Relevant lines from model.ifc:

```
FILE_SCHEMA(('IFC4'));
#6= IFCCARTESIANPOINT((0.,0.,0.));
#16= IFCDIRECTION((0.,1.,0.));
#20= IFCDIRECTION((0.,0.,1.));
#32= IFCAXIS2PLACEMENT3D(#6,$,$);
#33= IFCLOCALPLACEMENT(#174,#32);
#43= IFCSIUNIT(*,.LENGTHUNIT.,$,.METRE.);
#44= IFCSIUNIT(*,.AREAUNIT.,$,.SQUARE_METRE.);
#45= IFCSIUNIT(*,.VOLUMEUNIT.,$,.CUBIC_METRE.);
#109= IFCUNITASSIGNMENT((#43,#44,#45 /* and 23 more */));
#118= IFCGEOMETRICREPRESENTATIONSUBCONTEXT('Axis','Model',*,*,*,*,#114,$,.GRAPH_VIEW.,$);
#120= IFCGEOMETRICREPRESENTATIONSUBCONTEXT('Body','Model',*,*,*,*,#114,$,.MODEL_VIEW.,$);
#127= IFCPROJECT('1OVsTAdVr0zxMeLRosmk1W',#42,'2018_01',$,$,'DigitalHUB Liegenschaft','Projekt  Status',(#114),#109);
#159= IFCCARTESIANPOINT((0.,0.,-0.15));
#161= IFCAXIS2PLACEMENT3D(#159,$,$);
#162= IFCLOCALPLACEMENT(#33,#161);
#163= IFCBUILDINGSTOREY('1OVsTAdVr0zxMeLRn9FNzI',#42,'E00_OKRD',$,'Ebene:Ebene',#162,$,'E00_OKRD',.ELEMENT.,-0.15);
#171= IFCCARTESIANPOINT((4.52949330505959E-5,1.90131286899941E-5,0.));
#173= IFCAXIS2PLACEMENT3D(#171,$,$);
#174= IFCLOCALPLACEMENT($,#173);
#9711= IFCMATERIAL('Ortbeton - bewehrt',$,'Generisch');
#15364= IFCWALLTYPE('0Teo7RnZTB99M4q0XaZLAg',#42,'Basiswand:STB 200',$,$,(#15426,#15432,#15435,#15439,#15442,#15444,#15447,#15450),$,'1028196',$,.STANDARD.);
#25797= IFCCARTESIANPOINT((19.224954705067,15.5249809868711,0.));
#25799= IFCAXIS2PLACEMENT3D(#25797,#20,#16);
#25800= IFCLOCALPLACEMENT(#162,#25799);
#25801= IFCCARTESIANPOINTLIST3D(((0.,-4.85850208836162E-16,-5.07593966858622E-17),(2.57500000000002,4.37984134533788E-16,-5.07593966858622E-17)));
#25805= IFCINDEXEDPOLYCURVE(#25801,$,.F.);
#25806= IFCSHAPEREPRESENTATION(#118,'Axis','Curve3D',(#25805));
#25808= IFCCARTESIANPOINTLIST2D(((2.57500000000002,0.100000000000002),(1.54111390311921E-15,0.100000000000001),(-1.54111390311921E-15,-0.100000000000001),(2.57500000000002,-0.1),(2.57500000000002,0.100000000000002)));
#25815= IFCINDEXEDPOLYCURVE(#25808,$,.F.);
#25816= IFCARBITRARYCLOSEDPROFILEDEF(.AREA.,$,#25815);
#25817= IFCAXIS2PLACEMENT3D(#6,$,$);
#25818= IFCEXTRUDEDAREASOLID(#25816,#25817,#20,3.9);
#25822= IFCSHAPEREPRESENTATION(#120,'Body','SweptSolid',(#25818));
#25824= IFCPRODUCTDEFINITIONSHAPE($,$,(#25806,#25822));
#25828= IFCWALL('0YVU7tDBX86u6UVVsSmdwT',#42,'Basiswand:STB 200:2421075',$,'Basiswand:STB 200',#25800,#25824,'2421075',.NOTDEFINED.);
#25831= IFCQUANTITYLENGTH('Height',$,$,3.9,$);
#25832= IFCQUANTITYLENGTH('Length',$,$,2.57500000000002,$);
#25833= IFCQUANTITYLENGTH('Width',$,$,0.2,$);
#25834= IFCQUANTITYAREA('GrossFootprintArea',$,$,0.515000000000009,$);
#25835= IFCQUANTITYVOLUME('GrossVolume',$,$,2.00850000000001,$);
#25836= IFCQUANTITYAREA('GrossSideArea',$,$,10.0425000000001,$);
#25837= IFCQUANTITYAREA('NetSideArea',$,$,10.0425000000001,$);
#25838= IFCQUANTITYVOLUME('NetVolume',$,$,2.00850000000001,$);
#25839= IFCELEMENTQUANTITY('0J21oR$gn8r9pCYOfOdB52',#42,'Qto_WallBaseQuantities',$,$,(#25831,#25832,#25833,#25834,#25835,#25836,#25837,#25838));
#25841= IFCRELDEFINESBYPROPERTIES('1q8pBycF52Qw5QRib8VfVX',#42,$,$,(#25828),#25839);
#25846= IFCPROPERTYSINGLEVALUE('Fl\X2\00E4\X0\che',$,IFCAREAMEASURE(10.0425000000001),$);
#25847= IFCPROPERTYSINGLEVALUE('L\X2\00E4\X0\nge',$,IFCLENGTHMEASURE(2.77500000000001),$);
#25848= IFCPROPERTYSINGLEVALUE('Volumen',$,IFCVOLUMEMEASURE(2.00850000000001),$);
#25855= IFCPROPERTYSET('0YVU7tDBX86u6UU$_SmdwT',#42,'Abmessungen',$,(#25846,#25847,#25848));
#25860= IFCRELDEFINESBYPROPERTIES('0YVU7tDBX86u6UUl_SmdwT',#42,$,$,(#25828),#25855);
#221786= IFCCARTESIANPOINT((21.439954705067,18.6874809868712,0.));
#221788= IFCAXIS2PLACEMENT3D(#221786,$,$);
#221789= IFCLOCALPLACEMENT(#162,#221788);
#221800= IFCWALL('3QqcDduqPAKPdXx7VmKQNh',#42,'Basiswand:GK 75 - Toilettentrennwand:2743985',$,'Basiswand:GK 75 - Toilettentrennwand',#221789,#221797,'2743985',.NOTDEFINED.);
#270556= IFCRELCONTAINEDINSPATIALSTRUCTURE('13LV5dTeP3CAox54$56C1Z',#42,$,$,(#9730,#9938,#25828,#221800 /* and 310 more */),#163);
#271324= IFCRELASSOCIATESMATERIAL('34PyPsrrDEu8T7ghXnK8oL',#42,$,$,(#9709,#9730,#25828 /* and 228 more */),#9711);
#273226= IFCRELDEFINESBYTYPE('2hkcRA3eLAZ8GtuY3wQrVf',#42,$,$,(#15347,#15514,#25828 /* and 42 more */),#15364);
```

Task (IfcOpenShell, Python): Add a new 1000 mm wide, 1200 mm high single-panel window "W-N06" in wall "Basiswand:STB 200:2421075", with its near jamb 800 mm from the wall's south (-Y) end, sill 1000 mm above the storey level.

```python
import numpy as np
import ifcopenshell
import ifcopenshell.api.feature
import ifcopenshell.api.geometry
import ifcopenshell.api.pset
import ifcopenshell.api.root
import ifcopenshell.api.spatial
import ifcopenshell.geom
import ifcopenshell.util.element
import ifcopenshell.util.placement
import ifcopenshell.util.representation
import ifcopenshell.util.shape
import ifcopenshell.util.unit

model = ifcopenshell.open("model.ifc")
unit_scale = ifcopenshell.util.unit.calculate_unit_scale(model)
area_scale = ifcopenshell.util.unit.calculate_unit_scale(model, "AREAUNIT")
volume_scale = ifcopenshell.util.unit.calculate_unit_scale(model, "VOLUMEUNIT")
settings = ifcopenshell.geom.settings()


def volume(element):
    """Net volume in cubic metres, openings subtracted."""
    shape = ifcopenshell.geom.create_shape(settings, element)
    return ifcopenshell.util.shape.get_volume(shape.geometry)


wall = model.by_guid("0YVU7tDBX86u6UVVsSmdwT")
storey = ifcopenshell.util.element.get_container(wall, ifc_class="IfcBuildingStorey")
context = ifcopenshell.util.representation.get_context(model, "Model", "Body", "MODEL_VIEW")
before = volume(wall)

width, height, from_end, sill = 1, 1.2, 0.8, 1  # metres

# The wall runs along its own X axis, and the end named is its -X end.
wall_shape = ifcopenshell.geom.create_shape(settings, wall)
x, y, z = ifcopenshell.util.shape.get_vertices(wall_shape.geometry).T
start = x.min() + from_end
face, thickness = float(y.min()), float(y.max() - y.min())
wall_matrix = ifcopenshell.util.placement.get_local_placement(wall.ObjectPlacement)
level = ifcopenshell.util.placement.get_local_placement(storey.ObjectPlacement)[2, 3]


def in_wall(x, y):
    """Placement at x, y metres in the wall's axes, at sill height."""
    matrix = wall_matrix.copy()
    matrix[:, 3] = wall_matrix @ np.array([x / unit_scale, y / unit_scale, 0.0, 1.0])
    matrix[2, 3] = level + sill / unit_scale
    return matrix


# Opening: a box that overshoots both wall faces by 50 mm.
opening = ifcopenshell.api.root.create_entity(model, ifc_class="IfcOpeningElement", predefined_type="OPENING")
box = ifcopenshell.api.geometry.add_wall_representation(
    model, context=context, length=width, height=height, thickness=thickness + 0.1
)
ifcopenshell.api.geometry.assign_representation(model, product=opening, representation=box)
ifcopenshell.api.geometry.edit_object_placement(model, product=opening, matrix=in_wall(start, face - 0.05), is_si=False)
ifcopenshell.api.feature.add_feature(model, feature=opening, element=wall)

window = ifcopenshell.api.root.create_entity(model, ifc_class="IfcWindow", name="W-N06", predefined_type="WINDOW")
window.OverallWidth, window.OverallHeight = width / unit_scale, height / unit_scale
window.PartitioningType = "SINGLE_PANEL"
body = ifcopenshell.api.geometry.add_window_representation(
    model,
    context=context,
    overall_width=window.OverallWidth,
    overall_height=window.OverallHeight,
    partition_type="SINGLE_PANEL",
)
ifcopenshell.api.geometry.assign_representation(model, product=window, representation=body)
ifcopenshell.api.spatial.assign_container(model, products=[window], relating_structure=storey)
ifcopenshell.api.feature.add_filling(model, opening=opening, element=window)

# Centre the window in the wall's thickness.
ifcopenshell.api.geometry.edit_object_placement(model, product=window, matrix=in_wall(start, face), is_si=False)
window_shape = ifcopenshell.geom.create_shape(settings, window)
depth = ifcopenshell.util.shape.get_vertices(window_shape.geometry)[:, 1]
offset = face + thickness / 2 - (depth.min() + depth.max()) / 2
ifcopenshell.api.geometry.edit_object_placement(model, product=window, matrix=in_wall(start, offset), is_si=False)

after = volume(wall)

# Update the wall's stored quantities.
qto = model.by_id(ifcopenshell.util.element.get_pset(wall, "Qto_WallBaseQuantities", should_inherit=False)["id"])
ifcopenshell.api.pset.edit_qto(model, qto=qto, properties={
    "NetSideArea": after / thickness / area_scale,
    "NetVolume": after / volume_scale,
})
pset = model.by_id(ifcopenshell.util.element.get_pset(wall, "Abmessungen", should_inherit=False)["id"])
ifcopenshell.api.pset.edit_pset(model, pset=pset, properties={
    "Fläche": model.create_entity("IfcAreaMeasure", after / thickness / area_scale),
    "Volumen": model.create_entity("IfcVolumeMeasure", after / volume_scale),
})

print(f"wall volume {before:.3f} -> {after:.3f} m3")

model.write("model_v2.ifc")
```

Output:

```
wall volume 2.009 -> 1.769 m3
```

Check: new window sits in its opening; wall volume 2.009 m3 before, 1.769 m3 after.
